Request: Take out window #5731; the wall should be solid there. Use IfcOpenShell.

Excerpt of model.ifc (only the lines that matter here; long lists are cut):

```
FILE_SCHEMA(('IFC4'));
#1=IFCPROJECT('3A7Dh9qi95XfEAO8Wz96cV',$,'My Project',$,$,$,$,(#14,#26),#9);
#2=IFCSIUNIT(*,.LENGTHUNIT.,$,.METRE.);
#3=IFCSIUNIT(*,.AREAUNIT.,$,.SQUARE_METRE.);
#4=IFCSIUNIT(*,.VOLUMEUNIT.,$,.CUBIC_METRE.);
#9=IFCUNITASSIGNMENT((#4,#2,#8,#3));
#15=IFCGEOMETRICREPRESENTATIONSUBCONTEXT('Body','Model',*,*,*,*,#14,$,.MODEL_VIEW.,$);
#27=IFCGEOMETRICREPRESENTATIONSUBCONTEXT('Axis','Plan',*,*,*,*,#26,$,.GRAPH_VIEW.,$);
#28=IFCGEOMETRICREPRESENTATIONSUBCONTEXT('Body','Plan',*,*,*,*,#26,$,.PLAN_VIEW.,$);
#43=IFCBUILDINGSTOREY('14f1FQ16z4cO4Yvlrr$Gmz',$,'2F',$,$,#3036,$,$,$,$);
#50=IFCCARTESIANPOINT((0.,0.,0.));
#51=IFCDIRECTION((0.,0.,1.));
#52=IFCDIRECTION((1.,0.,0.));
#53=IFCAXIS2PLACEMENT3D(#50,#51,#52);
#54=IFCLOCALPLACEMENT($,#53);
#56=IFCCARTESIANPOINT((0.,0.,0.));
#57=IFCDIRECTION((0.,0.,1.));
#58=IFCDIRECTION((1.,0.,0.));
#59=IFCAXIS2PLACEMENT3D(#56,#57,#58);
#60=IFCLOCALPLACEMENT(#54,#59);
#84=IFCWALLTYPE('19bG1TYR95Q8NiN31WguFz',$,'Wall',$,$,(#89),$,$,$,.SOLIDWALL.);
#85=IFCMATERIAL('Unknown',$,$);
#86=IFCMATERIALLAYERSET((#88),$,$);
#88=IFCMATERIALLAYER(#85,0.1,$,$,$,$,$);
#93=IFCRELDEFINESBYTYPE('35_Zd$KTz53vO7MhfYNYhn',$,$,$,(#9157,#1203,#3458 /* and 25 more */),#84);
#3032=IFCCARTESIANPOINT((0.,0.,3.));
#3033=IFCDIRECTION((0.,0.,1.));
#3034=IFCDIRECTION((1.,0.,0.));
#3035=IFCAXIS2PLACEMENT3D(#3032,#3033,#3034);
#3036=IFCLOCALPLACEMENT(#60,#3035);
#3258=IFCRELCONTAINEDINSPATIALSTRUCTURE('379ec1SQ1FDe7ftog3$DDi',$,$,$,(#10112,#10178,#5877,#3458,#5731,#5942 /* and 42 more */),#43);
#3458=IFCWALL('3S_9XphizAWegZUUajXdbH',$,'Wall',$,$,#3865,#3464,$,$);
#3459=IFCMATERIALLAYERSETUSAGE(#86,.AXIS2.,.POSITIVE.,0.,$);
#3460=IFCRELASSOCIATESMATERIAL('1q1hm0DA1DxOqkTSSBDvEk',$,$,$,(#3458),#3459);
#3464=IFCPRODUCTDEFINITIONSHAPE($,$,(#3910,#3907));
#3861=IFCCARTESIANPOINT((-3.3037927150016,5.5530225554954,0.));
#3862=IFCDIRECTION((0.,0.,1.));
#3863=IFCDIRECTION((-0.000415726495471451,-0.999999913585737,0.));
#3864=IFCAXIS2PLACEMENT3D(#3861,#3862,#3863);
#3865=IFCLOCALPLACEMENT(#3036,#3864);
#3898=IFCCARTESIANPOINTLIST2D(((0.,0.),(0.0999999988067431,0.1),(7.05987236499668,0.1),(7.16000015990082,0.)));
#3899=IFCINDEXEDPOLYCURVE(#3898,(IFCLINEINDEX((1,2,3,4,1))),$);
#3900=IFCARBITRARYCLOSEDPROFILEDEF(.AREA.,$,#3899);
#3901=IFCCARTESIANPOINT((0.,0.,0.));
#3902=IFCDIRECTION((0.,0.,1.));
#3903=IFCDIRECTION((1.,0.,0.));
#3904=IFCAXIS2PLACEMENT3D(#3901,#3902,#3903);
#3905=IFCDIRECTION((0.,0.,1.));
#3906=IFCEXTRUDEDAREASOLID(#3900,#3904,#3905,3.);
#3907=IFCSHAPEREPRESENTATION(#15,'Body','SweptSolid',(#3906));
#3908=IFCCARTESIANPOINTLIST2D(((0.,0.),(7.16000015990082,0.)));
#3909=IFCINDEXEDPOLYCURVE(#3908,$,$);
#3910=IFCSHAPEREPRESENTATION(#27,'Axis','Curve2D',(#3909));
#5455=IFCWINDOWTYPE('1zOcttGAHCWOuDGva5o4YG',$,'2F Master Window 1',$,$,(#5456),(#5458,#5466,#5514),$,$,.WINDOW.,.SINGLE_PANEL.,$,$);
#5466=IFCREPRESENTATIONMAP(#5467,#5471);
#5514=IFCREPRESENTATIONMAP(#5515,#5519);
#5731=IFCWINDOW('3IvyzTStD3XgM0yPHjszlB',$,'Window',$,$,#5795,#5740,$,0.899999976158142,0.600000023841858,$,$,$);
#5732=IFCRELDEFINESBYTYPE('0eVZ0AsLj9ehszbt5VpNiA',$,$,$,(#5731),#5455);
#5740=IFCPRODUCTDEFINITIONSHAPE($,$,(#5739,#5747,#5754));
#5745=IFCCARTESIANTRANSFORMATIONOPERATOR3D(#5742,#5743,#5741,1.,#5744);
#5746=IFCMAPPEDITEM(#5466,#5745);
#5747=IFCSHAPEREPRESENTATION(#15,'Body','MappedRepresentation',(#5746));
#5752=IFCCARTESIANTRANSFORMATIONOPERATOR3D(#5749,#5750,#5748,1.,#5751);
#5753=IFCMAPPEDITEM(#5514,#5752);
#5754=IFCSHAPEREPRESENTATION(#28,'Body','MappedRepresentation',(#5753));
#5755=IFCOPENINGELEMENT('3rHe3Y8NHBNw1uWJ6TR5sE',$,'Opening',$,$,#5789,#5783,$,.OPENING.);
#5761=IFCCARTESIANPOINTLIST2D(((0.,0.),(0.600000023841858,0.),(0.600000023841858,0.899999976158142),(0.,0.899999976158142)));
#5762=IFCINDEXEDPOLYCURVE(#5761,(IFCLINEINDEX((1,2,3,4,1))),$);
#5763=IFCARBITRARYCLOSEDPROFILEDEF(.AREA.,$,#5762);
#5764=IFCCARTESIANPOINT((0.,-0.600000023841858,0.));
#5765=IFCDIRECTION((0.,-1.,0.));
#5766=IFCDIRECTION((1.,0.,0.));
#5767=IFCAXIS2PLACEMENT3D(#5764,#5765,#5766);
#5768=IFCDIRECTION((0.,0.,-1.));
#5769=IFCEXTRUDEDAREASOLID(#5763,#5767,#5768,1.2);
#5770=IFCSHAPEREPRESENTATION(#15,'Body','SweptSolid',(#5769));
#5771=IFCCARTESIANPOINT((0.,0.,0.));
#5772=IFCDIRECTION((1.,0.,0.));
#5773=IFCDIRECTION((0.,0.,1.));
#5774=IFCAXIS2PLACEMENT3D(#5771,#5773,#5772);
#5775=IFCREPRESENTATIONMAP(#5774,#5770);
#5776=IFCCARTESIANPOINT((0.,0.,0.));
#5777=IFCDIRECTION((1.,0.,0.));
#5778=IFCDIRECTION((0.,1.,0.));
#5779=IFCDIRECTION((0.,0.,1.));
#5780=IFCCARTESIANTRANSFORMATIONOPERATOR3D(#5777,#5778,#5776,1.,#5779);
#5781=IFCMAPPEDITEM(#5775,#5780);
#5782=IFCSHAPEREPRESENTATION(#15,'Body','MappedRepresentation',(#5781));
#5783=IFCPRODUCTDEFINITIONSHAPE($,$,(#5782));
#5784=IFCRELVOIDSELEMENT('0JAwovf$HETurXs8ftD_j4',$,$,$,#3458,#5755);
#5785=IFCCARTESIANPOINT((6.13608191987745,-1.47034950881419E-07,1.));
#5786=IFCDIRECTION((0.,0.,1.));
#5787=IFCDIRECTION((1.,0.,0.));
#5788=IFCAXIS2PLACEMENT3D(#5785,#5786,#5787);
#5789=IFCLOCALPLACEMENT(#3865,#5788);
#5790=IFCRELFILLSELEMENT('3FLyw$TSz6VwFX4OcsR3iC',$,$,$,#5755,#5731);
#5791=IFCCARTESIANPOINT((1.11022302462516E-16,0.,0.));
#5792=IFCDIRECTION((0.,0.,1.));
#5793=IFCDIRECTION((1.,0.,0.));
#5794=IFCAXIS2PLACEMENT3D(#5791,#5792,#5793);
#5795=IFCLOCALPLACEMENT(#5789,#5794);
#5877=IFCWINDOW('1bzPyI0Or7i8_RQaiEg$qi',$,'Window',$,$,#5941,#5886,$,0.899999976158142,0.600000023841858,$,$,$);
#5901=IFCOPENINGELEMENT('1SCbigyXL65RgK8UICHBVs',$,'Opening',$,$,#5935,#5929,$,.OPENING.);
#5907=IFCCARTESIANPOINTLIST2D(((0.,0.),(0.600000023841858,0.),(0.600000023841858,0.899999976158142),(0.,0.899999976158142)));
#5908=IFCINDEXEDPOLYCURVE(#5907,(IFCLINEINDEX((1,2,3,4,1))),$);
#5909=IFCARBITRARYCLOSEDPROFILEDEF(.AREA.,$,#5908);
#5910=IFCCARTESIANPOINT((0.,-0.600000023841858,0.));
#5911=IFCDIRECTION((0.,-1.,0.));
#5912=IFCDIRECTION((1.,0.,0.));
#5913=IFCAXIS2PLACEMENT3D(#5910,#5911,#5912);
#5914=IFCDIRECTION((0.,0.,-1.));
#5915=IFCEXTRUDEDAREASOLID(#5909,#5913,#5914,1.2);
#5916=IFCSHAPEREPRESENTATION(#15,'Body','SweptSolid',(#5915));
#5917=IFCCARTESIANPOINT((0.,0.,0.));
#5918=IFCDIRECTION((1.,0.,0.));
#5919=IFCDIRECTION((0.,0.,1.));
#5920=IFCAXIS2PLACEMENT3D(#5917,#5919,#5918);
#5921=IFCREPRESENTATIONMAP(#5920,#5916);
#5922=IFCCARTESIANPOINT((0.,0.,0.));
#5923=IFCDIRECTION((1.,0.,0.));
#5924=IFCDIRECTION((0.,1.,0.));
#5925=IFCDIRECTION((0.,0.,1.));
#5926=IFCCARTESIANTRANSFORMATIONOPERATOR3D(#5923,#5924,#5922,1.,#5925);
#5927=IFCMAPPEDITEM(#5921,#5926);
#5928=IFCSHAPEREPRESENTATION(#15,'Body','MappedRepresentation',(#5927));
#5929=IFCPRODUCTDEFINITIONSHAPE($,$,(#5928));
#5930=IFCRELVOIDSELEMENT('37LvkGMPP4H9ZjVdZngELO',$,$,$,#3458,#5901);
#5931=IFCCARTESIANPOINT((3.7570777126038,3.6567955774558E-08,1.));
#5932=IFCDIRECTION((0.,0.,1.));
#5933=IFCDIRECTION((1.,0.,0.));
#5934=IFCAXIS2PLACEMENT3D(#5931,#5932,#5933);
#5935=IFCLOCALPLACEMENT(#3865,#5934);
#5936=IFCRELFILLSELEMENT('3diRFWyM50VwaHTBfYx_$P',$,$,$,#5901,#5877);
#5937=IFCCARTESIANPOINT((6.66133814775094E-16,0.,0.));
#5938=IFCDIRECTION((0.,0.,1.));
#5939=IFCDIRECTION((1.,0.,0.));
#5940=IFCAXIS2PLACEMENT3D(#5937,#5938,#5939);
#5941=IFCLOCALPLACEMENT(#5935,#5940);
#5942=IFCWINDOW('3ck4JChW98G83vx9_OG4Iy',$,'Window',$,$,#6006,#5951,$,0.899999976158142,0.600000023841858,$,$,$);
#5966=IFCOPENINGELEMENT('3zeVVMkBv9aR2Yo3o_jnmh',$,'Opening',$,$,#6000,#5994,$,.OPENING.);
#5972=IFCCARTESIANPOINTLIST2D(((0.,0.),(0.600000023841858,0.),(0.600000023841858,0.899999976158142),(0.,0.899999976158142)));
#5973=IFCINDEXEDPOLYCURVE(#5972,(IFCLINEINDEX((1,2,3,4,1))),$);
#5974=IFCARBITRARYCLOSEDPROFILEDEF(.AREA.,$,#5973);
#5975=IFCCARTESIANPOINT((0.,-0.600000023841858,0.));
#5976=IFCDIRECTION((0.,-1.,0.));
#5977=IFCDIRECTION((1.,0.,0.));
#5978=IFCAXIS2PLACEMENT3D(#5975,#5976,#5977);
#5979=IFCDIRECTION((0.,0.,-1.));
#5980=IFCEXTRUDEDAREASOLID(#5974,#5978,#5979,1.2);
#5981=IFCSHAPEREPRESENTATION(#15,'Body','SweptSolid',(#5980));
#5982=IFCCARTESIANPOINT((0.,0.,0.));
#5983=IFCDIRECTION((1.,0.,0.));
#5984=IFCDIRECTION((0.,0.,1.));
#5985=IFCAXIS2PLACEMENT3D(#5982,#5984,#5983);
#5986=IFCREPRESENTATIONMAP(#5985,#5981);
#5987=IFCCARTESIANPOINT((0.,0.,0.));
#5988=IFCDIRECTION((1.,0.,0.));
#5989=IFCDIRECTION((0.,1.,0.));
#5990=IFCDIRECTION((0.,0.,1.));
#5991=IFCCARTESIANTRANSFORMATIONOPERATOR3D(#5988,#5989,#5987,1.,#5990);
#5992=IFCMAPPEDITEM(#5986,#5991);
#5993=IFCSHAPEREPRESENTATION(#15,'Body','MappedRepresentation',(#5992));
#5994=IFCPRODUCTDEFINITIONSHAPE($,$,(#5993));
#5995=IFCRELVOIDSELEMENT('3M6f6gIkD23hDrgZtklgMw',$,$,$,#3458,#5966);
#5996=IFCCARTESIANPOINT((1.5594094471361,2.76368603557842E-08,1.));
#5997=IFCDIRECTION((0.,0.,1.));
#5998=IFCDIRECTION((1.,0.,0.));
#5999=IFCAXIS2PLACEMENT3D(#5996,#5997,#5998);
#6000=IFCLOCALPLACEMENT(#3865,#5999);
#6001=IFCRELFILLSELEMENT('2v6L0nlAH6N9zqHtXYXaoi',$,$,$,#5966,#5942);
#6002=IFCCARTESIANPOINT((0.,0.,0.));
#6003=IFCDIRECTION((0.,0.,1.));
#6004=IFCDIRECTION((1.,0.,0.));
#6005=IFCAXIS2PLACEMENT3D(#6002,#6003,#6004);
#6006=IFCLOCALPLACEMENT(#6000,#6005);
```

```python
import ifcopenshell
import ifcopenshell.api.feature
import ifcopenshell.api.root
import ifcopenshell.geom
import ifcopenshell.util.shape

model = ifcopenshell.open("model.ifc")
settings = ifcopenshell.geom.settings()


def volume(element):
    """Net volume in cubic metres, openings subtracted."""
    shape = ifcopenshell.geom.create_shape(settings, element)
    return ifcopenshell.util.shape.get_volume(shape.geometry)


window = model.by_guid("3IvyzTStD3XgM0yPHjszlB")
opening = window.FillsVoids[0].RelatingOpeningElement
wall = opening.VoidsElements[0].RelatingBuildingElement
before = volume(wall)

ifcopenshell.api.root.remove_product(model, product=window)
ifcopenshell.api.feature.remove_feature(model, feature=opening)

after = volume(wall)

print(f"wall volume {before:.3f} -> {after:.3f} m3")

model.write("model_rev.ifc")
```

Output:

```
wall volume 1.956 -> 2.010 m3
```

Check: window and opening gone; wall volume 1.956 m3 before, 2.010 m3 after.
